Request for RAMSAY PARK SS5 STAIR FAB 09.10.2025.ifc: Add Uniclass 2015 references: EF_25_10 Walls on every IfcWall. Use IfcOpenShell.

First a look at what the model holds.

```python
import ifcopenshell

model = ifcopenshell.open("RAMSAY PARK SS5 STAIR FAB 09.10.2025.ifc")
print(model.schema)
print("classifications:", [c.Name for c in model.by_type("IfcClassification")])
for ifc_class in ("IfcDoor", "IfcRoof", "IfcStair", "IfcWall", "IfcWindow"):
    print(ifc_class, len(model.by_type(ifc_class)))
```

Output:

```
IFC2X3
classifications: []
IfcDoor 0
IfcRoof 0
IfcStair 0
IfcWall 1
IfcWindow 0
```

```python
import ifcopenshell
import ifcopenshell.api.classification

model = ifcopenshell.open("RAMSAY PARK SS5 STAIR FAB 09.10.2025.ifc")

# IFC2X3 requires Source and Edition and has no link from the project to the system.
system = model.create_entity("IfcClassification", Source="NBS", Edition="2015", Name="Uniclass 2015")

codes = {
    "IfcWall": ("EF_25_10", "Walls"),
}
for ifc_class, (code, name) in codes.items():
    products = model.by_type(ifc_class)
    ifcopenshell.api.classification.add_reference(
        model, products=products, classification=system, identification=code, name=name
    )
    print(code, len(products))

model.write("RAMSAY PARK SS5 STAIR FAB 09.10.2025_edited.ifc")
```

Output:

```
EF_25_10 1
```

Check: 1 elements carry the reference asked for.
